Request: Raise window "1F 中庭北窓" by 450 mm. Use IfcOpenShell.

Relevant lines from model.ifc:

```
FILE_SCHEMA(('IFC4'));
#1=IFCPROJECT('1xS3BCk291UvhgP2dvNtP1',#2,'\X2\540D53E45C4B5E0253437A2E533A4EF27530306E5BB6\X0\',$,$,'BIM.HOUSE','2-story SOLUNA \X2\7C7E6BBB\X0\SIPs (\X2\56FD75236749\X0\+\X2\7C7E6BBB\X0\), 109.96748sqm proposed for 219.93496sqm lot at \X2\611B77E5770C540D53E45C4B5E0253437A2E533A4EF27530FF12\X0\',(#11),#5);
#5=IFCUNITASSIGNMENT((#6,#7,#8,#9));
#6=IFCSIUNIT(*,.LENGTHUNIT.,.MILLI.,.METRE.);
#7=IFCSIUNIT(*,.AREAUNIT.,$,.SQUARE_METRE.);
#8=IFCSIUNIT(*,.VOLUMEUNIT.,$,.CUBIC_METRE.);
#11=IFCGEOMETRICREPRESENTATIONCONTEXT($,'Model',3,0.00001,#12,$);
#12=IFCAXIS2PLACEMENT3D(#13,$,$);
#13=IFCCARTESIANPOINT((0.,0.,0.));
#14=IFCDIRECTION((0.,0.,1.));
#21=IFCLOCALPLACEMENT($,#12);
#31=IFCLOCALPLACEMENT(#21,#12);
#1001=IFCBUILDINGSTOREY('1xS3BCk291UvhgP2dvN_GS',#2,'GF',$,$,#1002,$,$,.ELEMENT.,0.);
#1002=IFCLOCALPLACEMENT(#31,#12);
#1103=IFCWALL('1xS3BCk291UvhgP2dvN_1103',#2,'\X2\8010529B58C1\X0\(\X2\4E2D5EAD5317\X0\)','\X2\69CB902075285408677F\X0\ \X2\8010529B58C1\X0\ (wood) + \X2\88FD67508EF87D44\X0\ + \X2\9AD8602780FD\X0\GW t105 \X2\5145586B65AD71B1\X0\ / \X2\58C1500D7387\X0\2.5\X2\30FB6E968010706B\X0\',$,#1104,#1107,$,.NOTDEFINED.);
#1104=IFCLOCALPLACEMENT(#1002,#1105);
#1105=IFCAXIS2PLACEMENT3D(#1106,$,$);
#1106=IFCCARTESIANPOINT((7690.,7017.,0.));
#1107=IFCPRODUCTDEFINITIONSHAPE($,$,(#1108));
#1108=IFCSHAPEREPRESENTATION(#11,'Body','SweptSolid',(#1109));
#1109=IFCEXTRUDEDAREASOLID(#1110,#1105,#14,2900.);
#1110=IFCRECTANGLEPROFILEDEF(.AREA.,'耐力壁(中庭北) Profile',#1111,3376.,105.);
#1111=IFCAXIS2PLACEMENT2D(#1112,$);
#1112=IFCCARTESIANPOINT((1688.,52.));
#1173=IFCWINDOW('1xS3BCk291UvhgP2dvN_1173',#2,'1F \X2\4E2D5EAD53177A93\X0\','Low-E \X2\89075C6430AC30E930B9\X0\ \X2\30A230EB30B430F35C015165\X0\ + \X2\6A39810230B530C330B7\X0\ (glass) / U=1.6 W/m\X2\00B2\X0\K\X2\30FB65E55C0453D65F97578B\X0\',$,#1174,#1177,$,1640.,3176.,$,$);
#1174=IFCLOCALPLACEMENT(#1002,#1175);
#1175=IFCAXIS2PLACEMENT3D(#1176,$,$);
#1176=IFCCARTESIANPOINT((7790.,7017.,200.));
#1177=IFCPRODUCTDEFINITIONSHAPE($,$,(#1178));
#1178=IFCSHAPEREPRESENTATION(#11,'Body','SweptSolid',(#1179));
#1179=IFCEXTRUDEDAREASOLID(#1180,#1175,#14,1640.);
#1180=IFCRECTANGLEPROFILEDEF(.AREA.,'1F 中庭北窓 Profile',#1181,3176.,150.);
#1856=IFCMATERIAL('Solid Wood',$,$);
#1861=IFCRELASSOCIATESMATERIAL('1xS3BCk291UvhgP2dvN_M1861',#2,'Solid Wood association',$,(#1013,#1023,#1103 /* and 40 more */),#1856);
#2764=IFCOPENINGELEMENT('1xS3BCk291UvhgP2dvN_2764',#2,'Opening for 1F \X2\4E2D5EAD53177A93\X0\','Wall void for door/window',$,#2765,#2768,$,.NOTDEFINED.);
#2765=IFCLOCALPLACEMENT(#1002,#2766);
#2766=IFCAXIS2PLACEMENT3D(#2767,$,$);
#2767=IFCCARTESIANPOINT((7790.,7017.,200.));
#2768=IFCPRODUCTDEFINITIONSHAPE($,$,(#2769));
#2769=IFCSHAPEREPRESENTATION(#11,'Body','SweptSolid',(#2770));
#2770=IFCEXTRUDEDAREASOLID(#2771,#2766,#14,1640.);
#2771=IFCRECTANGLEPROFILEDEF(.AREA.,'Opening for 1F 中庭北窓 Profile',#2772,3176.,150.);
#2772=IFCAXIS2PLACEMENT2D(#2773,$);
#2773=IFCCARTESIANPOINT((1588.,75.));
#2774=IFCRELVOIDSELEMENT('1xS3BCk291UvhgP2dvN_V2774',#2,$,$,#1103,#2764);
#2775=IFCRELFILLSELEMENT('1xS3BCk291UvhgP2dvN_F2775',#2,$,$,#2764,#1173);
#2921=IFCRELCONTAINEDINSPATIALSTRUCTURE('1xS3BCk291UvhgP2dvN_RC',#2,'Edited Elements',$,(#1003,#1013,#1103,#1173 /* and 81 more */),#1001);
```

```python
import numpy as np
import ifcopenshell
import ifcopenshell.api.geometry
import ifcopenshell.util.placement
import ifcopenshell.util.unit

model = ifcopenshell.open("model.ifc")
unit_scale = ifcopenshell.util.unit.calculate_unit_scale(model)

window = model.by_id(1173)
opening = window.FillsVoids[0].RelatingOpeningElement
dz = 0.45 / unit_scale

shift = np.array([0.0, 0.0, dz])
# The window is not placed relative to its opening, so move both.
for product in (opening, window):
    matrix = ifcopenshell.util.placement.get_local_placement(product.ObjectPlacement)
    matrix[:3, 3] += shift
    ifcopenshell.api.geometry.edit_object_placement(model, product=product, matrix=matrix, is_si=False)

print(f"moved by {dz * unit_scale:+.3f} m")

model.write("model_updated.ifc")
```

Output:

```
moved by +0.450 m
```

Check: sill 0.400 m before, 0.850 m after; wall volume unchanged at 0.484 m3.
